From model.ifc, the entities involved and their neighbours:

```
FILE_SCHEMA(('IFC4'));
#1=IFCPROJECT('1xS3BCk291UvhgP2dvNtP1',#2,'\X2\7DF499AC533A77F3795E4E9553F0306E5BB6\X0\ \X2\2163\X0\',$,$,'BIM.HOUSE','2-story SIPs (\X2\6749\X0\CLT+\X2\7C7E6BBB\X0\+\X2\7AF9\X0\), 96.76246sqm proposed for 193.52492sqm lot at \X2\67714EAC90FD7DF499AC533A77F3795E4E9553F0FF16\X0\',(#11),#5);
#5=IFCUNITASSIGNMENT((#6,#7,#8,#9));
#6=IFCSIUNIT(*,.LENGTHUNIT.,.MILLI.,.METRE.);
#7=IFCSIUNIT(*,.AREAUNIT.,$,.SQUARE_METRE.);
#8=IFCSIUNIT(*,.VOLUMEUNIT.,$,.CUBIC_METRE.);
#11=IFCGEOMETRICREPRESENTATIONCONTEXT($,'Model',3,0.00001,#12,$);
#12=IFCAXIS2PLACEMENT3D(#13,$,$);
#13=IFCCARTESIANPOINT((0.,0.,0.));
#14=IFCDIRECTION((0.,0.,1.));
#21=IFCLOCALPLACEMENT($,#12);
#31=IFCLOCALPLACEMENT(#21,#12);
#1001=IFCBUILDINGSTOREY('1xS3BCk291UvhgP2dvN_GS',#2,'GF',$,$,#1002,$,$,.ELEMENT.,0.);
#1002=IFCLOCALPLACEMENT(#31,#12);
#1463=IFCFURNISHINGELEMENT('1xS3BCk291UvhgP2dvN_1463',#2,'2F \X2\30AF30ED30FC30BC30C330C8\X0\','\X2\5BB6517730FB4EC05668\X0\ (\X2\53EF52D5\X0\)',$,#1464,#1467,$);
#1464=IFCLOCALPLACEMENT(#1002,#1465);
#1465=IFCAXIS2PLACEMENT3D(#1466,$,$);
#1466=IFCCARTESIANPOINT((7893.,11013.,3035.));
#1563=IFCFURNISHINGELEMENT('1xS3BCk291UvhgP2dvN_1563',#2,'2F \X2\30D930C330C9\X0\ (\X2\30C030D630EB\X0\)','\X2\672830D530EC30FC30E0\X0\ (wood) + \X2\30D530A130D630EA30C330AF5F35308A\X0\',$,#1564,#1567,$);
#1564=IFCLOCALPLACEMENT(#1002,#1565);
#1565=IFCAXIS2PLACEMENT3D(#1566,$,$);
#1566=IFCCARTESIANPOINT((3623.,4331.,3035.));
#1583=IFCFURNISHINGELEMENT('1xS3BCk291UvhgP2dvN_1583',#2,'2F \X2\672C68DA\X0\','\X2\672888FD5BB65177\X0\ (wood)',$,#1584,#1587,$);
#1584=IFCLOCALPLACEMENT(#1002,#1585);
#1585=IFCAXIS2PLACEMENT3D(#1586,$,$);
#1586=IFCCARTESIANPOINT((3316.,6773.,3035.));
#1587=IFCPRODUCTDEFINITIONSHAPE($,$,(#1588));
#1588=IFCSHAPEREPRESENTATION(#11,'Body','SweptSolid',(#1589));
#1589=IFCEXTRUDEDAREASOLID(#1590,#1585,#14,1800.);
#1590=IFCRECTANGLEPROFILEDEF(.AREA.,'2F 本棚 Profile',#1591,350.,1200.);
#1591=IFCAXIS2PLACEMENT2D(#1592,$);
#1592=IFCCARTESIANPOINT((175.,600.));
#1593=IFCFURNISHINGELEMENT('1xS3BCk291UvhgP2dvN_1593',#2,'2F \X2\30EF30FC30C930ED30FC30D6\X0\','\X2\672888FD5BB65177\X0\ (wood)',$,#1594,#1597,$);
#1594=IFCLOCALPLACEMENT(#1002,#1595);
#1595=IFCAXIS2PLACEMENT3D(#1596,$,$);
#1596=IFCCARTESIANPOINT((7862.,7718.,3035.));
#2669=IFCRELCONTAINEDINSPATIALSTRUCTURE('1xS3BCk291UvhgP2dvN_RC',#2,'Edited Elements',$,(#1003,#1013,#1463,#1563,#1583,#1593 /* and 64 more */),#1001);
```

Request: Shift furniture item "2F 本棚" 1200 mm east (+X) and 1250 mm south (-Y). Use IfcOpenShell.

```python
import ifcopenshell
import ifcopenshell.api.geometry
import ifcopenshell.util.placement

model = ifcopenshell.open("model.ifc")

item = model.by_guid("1xS3BCk291UvhgP2dvN_1583")
matrix = ifcopenshell.util.placement.get_local_placement(item.ObjectPlacement)
matrix[0, 3] += 1200.0
matrix[1, 3] -= 1250.0
ifcopenshell.api.geometry.edit_object_placement(model, product=item, matrix=matrix, is_si=False)

print(ifcopenshell.util.placement.get_local_placement(item.ObjectPlacement).round(3) + 0.0)

model.write("model-out.ifc")
```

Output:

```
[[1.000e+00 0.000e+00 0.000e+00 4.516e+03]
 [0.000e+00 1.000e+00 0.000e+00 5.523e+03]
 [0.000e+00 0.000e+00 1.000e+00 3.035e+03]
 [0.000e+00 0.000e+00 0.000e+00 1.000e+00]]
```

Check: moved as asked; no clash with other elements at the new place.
